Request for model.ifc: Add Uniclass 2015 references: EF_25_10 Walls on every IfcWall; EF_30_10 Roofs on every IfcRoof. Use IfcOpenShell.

First a look at what the model holds.

```python
import ifcopenshell

model = ifcopenshell.open("model.ifc")
print(model.schema)
print("classifications:", [c.Name for c in model.by_type("IfcClassification")])
for ifc_class in ("IfcDoor", "IfcRoof", "IfcStair", "IfcWall", "IfcWindow"):
    print(ifc_class, len(model.by_type(ifc_class)))
```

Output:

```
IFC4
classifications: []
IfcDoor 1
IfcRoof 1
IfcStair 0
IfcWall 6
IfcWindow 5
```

```python
import ifcopenshell
import ifcopenshell.api.classification

model = ifcopenshell.open("model.ifc")

system = ifcopenshell.api.classification.add_classification(model, classification="Uniclass 2015")

codes = {
    "IfcWall": ("EF_25_10", "Walls"),
    "IfcRoof": ("EF_30_10", "Roofs"),
}
for ifc_class, (code, name) in codes.items():
    products = model.by_type(ifc_class)
    ifcopenshell.api.classification.add_reference(
        model, products=products, classification=system, identification=code, name=name
    )
    print(code, len(products))

model.write("model_v2.ifc")
```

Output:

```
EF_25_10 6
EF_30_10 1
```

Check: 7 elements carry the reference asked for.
